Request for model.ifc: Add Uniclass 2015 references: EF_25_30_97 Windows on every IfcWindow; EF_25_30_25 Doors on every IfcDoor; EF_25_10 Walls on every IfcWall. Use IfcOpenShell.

First a look at what the model holds.

```python
import ifcopenshell

model = ifcopenshell.open("model.ifc")
print(model.schema)
print("classifications:", [c.Name for c in model.by_type("IfcClassification")])
for ifc_class in ("IfcDoor", "IfcRoof", "IfcStair", "IfcWall", "IfcWindow"):
    print(ifc_class, len(model.by_type(ifc_class)))
```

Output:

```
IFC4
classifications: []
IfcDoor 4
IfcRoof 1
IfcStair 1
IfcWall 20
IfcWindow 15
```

```python
import ifcopenshell
import ifcopenshell.api.classification

model = ifcopenshell.open("model.ifc")

system = ifcopenshell.api.classification.add_classification(model, classification="Uniclass 2015")

codes = {
    "IfcWindow": ("EF_25_30_97", "Windows"),
    "IfcDoor": ("EF_25_30_25", "Doors"),
    "IfcWall": ("EF_25_10", "Walls"),
}
for ifc_class, (code, name) in codes.items():
    products = model.by_type(ifc_class)
    ifcopenshell.api.classification.add_reference(
        model, products=products, classification=system, identification=code, name=name
    )
    print(code, len(products))

model.write("model_v2.ifc")
```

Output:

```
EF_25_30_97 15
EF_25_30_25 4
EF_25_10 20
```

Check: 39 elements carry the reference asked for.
